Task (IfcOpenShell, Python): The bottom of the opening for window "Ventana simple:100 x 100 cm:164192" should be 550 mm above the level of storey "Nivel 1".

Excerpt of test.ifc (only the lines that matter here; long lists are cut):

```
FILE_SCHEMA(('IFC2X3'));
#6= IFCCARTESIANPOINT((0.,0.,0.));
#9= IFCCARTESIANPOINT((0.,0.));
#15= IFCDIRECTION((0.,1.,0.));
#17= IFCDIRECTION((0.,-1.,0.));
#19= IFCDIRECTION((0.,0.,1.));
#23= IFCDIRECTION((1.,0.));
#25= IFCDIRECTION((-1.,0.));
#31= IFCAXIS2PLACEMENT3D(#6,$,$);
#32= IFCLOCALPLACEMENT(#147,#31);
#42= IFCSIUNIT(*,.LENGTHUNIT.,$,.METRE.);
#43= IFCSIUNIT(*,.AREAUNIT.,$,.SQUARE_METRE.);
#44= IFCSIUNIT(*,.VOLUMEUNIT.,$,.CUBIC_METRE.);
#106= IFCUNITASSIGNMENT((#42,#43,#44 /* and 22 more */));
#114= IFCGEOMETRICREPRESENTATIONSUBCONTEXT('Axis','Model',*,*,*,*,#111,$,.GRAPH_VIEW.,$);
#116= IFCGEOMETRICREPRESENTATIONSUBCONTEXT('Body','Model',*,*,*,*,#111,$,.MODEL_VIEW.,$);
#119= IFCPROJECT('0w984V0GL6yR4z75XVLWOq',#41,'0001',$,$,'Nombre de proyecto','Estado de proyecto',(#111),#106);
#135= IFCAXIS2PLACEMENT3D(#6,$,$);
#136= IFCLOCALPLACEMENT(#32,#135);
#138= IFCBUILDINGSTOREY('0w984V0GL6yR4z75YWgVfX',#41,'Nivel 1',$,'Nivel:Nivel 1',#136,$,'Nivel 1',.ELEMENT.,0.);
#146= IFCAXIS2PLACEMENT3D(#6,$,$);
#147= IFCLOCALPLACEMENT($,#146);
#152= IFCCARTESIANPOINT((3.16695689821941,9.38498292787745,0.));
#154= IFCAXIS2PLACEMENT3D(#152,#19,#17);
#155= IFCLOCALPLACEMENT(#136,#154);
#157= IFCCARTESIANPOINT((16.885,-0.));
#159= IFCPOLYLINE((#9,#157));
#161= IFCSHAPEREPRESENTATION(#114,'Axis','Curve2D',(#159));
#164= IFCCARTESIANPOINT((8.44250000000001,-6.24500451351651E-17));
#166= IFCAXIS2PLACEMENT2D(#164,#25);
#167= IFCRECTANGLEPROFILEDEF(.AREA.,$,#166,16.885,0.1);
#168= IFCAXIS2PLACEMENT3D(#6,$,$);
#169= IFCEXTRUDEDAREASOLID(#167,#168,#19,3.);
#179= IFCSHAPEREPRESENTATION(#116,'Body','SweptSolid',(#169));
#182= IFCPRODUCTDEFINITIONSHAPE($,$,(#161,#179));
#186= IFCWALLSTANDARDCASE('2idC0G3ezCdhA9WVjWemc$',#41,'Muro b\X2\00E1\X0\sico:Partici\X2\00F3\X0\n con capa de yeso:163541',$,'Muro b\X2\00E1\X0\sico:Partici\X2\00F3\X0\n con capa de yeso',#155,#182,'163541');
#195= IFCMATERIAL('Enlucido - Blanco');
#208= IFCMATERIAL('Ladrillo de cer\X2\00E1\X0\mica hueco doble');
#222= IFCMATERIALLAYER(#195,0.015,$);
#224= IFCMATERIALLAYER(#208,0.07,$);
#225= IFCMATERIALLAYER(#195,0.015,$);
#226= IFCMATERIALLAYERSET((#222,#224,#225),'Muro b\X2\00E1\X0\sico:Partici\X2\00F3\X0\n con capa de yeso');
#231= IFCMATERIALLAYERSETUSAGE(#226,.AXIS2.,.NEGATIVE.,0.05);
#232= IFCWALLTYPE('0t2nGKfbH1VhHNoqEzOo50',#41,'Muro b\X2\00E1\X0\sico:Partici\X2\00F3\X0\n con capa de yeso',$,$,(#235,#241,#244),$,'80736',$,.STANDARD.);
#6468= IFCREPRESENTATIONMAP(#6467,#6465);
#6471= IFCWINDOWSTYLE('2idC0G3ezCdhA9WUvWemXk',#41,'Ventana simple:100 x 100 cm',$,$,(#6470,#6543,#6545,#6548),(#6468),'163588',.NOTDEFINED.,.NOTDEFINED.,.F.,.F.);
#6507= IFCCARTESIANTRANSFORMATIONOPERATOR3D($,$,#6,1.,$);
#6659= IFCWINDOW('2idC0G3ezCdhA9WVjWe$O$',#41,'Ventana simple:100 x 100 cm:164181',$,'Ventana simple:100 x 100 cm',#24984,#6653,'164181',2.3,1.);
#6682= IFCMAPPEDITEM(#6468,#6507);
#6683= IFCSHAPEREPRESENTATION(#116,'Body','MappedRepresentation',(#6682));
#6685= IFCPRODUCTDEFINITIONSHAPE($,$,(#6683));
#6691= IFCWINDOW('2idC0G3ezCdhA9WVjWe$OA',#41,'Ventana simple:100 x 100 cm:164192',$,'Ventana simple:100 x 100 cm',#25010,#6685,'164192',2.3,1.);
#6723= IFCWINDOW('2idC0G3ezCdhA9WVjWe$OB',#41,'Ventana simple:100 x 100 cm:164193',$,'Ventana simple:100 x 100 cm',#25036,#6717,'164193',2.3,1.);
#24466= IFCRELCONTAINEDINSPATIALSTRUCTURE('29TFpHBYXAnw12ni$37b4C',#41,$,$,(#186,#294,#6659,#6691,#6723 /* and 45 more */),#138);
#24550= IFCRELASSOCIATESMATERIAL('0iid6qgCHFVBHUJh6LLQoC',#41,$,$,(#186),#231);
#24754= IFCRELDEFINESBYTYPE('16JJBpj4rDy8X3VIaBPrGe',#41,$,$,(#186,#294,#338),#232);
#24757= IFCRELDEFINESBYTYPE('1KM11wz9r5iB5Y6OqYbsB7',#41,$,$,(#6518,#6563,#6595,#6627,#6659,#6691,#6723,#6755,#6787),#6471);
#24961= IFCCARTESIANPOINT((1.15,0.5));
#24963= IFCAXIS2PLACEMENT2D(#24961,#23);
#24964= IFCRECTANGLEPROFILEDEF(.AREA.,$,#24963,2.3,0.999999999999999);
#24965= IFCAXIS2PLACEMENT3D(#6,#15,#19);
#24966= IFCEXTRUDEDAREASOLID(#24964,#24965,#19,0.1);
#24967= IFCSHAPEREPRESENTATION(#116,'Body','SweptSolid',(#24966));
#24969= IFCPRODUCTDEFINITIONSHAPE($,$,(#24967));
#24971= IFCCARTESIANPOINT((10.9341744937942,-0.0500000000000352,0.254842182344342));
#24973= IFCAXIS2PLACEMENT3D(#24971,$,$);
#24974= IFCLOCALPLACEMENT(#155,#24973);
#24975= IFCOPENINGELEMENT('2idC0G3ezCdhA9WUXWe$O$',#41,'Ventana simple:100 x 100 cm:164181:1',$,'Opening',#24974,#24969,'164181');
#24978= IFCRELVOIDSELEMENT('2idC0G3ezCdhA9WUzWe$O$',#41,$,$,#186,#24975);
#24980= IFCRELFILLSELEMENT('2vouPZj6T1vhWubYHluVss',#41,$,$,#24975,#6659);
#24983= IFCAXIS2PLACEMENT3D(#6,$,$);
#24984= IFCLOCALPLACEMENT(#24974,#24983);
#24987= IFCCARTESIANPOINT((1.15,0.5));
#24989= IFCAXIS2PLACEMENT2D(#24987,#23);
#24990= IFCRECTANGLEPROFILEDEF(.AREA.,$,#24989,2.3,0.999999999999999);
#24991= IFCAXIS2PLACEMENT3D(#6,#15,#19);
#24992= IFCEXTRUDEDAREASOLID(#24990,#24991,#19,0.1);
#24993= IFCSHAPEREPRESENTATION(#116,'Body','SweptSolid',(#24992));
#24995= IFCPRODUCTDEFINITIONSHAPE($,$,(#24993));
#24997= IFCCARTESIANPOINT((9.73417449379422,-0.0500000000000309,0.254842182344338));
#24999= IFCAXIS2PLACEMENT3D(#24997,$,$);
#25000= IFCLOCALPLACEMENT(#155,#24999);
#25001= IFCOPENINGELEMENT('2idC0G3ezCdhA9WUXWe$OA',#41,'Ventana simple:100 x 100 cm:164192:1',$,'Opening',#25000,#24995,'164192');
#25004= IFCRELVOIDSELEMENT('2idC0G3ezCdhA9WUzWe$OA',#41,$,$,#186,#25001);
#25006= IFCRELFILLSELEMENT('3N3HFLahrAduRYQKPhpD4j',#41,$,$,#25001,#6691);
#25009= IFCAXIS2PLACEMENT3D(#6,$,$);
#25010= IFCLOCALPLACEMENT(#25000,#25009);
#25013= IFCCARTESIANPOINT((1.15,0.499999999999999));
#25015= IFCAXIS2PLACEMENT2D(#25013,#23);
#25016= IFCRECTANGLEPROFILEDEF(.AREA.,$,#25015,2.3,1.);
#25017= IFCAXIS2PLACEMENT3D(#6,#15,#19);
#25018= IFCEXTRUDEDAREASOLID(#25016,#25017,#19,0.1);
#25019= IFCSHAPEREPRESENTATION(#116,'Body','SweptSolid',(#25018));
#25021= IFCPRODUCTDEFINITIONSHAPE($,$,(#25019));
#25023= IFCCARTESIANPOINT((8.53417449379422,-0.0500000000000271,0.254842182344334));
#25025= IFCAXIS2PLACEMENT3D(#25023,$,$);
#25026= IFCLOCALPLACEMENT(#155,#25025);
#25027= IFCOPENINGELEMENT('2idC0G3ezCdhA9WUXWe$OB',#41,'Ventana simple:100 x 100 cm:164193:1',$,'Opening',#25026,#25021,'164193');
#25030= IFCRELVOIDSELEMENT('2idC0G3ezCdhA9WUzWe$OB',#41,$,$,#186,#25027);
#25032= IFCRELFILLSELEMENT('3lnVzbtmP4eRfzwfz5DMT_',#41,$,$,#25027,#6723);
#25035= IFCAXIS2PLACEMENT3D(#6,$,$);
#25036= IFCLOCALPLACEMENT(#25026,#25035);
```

```python
import numpy as np
import ifcopenshell
import ifcopenshell.api.geometry
import ifcopenshell.geom
import ifcopenshell.util.element
import ifcopenshell.util.placement
import ifcopenshell.util.shape
import ifcopenshell.util.unit

model = ifcopenshell.open("test.ifc")
unit_scale = ifcopenshell.util.unit.calculate_unit_scale(model)

window = model.by_id(6691)
opening = window.FillsVoids[0].RelatingOpeningElement
storey = ifcopenshell.util.element.get_container(window, ifc_class="IfcBuildingStorey")
level = ifcopenshell.util.placement.get_local_placement(storey.ObjectPlacement)[2, 3]

# The opening's origin need not be at the sill, so measure its lowest point.
shape = ifcopenshell.geom.create_shape(ifcopenshell.geom.settings(), opening)
bottom = ifcopenshell.util.shape.get_shape_bottom_elevation(shape, shape.geometry) / unit_scale
dz = level + 0.55 / unit_scale - bottom

shift = np.array([0.0, 0.0, dz])
# The window is placed relative to its opening, so it follows when the opening moves.
matrix = ifcopenshell.util.placement.get_local_placement(opening.ObjectPlacement)
matrix[:3, 3] += shift
ifcopenshell.api.geometry.edit_object_placement(
    model, product=opening, matrix=matrix, is_si=False, should_transform_children=True
)

print(f"moved by {dz * unit_scale:+.3f} m")

model.write("test-out.ifc")
```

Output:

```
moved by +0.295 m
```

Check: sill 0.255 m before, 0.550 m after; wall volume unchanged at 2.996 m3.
